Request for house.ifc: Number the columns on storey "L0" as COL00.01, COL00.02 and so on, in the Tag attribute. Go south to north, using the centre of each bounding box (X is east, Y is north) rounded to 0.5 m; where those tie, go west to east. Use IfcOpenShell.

First a look at what the model holds.

```python
import ifcopenshell
import ifcopenshell.util.element
import ifcopenshell.util.placement

model = ifcopenshell.open("house.ifc")
print(model.schema)
storey = next(s for s in model.by_type("IfcBuildingStorey") if s.Name == "L0")
columns = [e for e in ifcopenshell.util.element.get_decomposition(storey) if e.is_a("IfcColumn")]
for e in sorted(columns, key=lambda e: e.id()):
    origin = ifcopenshell.util.placement.get_local_placement(e.ObjectPlacement)[:3, 3]
    print(e.id(), e.Tag, e.Name, origin.round(2) + 0.0, sep=" | ")
```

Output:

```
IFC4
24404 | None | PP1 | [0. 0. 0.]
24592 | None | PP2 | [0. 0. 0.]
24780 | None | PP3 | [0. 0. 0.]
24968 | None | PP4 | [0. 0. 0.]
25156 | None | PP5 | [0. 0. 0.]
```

```python
import ifcopenshell
import ifcopenshell.geom
import ifcopenshell.util.element
import ifcopenshell.util.shape

model = ifcopenshell.open("house.ifc")
settings = ifcopenshell.geom.settings()
settings.set("use-world-coords", True)


def centre(element):
    shape = ifcopenshell.geom.create_shape(settings, element)
    return ifcopenshell.util.shape.get_bbox_centroid(shape.geometry)


storey = next(s for s in model.by_type("IfcBuildingStorey") if s.Name == "L0")
columns = [e for e in ifcopenshell.util.element.get_decomposition(storey) if e.is_a("IfcColumn")]

# Insertion points can sit at a corner or the storey origin, so sort by the geometry (in metres).
centres = {e: centre(e) for e in columns}
columns.sort(key=lambda e: (round(centres[e][1] / 0.5), centres[e][0]))

for i, e in enumerate(columns, start=1):
    number = f"COL00.{i:02d}"
    e.Tag = number
    print(e.id(), number)

model.write("house_edited.ifc")
```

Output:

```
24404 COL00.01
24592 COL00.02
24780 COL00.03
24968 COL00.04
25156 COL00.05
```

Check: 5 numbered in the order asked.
